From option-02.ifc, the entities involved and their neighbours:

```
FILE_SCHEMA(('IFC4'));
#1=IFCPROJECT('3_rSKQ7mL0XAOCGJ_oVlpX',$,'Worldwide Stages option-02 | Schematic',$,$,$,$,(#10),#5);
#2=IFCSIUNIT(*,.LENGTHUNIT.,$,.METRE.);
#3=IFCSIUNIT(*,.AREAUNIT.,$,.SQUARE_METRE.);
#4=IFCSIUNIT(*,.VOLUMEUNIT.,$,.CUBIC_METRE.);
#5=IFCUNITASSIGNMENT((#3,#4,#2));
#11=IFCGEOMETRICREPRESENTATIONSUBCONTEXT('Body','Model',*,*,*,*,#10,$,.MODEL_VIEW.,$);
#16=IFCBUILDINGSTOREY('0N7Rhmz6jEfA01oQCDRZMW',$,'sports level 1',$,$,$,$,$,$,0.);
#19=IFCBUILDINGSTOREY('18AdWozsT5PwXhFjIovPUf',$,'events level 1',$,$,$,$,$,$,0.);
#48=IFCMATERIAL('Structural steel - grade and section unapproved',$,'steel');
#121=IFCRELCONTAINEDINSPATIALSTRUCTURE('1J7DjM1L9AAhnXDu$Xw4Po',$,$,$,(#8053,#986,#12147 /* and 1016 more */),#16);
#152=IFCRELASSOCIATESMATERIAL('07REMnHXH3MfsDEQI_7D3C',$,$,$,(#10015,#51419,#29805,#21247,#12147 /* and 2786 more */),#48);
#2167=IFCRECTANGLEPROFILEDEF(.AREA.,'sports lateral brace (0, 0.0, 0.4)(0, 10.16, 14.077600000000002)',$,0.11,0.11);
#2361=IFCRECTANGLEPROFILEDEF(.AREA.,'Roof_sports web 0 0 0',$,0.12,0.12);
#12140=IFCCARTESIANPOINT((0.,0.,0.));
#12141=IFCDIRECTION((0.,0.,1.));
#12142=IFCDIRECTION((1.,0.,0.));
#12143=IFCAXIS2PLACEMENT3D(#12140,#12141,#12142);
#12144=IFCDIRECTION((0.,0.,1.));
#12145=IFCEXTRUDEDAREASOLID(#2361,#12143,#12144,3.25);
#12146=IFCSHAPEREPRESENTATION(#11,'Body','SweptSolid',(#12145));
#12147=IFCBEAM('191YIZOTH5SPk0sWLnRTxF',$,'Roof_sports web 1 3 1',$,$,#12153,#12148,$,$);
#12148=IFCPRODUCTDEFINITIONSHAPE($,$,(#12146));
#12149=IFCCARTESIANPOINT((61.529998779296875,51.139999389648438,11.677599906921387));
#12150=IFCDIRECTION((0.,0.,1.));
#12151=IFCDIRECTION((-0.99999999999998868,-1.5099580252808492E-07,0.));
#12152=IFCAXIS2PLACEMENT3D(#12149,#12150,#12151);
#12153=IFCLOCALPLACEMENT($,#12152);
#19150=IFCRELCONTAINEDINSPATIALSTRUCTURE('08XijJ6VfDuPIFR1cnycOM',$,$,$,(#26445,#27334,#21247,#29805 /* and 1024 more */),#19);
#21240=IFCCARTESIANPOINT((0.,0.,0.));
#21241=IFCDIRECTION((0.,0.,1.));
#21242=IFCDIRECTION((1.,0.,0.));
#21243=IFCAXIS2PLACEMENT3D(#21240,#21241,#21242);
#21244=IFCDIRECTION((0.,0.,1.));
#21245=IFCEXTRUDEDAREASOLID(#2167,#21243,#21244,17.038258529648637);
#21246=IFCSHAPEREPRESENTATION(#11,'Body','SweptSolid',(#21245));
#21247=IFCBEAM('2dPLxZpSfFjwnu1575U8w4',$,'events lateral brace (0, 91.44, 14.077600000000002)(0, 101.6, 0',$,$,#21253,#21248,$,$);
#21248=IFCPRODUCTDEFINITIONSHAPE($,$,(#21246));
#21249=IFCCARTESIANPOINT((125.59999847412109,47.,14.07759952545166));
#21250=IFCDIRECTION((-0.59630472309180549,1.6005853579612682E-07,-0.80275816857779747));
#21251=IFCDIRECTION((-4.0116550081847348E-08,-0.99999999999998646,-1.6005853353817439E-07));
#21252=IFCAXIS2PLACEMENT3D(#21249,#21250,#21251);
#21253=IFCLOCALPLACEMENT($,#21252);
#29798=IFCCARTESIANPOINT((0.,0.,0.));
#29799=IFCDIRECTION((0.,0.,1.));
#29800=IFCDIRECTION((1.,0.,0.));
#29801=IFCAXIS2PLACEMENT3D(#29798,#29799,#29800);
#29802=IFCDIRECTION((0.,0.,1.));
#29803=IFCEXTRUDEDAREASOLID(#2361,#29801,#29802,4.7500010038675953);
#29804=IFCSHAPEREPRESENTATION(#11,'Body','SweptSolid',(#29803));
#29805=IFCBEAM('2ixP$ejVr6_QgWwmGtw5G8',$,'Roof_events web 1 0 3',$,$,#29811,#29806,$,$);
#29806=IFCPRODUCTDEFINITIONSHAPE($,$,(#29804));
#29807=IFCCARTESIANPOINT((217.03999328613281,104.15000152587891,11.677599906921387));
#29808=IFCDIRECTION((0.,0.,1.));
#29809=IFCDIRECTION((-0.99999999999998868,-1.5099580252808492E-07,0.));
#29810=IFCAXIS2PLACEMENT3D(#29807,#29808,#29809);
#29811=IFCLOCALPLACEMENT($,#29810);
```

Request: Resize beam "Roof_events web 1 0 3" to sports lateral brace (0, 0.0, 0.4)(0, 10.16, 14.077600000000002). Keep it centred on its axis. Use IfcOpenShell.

```python
import ifcopenshell
import ifcopenshell.util.element
import ifcopenshell.util.representation

model = ifcopenshell.open("option-02.ifc")

member = model.by_id(29805)
source = next(p for p in model.by_type("IfcRectangleProfileDef") if p.ProfileName == "sports lateral brace (0, 0.0, 0.4)(0, 10.16, 14.077600000000002)")

body = ifcopenshell.util.representation.get_representation(member, "Model", "Body")
solid = body.Items[0]
old_profile = solid.SweptArea

# Copy the section's sizes but keep this member's own profile position.
profile = ifcopenshell.util.element.copy(model, source)
profile.Position = old_profile.Position
solid.SweptArea = profile
if not model.get_total_inverses(old_profile):
    ifcopenshell.util.element.remove_deep2(model, old_profile)

print(solid.SweptArea)

model.write("option-02_edited.ifc")
```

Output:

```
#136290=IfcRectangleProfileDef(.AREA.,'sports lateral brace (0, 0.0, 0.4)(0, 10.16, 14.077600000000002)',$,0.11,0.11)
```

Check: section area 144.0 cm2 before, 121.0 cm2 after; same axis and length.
